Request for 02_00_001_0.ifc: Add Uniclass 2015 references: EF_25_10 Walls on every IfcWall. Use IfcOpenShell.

First a look at what the model holds.

```python
import ifcopenshell

model = ifcopenshell.open("02_00_001_0.ifc")
print(model.schema)
print("classifications:", [c.Name for c in model.by_type("IfcClassification")])
for ifc_class in ("IfcDoor", "IfcRoof", "IfcStair", "IfcWall", "IfcWindow"):
    print(ifc_class, len(model.by_type(ifc_class)))
```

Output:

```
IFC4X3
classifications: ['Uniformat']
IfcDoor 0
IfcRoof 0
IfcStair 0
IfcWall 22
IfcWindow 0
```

```python
import ifcopenshell
import ifcopenshell.api.classification

model = ifcopenshell.open("02_00_001_0.ifc")

system = ifcopenshell.api.classification.add_classification(model, classification="Uniclass 2015")

codes = {
    "IfcWall": ("EF_25_10", "Walls"),
}
for ifc_class, (code, name) in codes.items():
    products = model.by_type(ifc_class)
    ifcopenshell.api.classification.add_reference(
        model, products=products, classification=system, identification=code, name=name
    )
    print(code, len(products))

model.write("02_00_001_0_rev.ifc")
```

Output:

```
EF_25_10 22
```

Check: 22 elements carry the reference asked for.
